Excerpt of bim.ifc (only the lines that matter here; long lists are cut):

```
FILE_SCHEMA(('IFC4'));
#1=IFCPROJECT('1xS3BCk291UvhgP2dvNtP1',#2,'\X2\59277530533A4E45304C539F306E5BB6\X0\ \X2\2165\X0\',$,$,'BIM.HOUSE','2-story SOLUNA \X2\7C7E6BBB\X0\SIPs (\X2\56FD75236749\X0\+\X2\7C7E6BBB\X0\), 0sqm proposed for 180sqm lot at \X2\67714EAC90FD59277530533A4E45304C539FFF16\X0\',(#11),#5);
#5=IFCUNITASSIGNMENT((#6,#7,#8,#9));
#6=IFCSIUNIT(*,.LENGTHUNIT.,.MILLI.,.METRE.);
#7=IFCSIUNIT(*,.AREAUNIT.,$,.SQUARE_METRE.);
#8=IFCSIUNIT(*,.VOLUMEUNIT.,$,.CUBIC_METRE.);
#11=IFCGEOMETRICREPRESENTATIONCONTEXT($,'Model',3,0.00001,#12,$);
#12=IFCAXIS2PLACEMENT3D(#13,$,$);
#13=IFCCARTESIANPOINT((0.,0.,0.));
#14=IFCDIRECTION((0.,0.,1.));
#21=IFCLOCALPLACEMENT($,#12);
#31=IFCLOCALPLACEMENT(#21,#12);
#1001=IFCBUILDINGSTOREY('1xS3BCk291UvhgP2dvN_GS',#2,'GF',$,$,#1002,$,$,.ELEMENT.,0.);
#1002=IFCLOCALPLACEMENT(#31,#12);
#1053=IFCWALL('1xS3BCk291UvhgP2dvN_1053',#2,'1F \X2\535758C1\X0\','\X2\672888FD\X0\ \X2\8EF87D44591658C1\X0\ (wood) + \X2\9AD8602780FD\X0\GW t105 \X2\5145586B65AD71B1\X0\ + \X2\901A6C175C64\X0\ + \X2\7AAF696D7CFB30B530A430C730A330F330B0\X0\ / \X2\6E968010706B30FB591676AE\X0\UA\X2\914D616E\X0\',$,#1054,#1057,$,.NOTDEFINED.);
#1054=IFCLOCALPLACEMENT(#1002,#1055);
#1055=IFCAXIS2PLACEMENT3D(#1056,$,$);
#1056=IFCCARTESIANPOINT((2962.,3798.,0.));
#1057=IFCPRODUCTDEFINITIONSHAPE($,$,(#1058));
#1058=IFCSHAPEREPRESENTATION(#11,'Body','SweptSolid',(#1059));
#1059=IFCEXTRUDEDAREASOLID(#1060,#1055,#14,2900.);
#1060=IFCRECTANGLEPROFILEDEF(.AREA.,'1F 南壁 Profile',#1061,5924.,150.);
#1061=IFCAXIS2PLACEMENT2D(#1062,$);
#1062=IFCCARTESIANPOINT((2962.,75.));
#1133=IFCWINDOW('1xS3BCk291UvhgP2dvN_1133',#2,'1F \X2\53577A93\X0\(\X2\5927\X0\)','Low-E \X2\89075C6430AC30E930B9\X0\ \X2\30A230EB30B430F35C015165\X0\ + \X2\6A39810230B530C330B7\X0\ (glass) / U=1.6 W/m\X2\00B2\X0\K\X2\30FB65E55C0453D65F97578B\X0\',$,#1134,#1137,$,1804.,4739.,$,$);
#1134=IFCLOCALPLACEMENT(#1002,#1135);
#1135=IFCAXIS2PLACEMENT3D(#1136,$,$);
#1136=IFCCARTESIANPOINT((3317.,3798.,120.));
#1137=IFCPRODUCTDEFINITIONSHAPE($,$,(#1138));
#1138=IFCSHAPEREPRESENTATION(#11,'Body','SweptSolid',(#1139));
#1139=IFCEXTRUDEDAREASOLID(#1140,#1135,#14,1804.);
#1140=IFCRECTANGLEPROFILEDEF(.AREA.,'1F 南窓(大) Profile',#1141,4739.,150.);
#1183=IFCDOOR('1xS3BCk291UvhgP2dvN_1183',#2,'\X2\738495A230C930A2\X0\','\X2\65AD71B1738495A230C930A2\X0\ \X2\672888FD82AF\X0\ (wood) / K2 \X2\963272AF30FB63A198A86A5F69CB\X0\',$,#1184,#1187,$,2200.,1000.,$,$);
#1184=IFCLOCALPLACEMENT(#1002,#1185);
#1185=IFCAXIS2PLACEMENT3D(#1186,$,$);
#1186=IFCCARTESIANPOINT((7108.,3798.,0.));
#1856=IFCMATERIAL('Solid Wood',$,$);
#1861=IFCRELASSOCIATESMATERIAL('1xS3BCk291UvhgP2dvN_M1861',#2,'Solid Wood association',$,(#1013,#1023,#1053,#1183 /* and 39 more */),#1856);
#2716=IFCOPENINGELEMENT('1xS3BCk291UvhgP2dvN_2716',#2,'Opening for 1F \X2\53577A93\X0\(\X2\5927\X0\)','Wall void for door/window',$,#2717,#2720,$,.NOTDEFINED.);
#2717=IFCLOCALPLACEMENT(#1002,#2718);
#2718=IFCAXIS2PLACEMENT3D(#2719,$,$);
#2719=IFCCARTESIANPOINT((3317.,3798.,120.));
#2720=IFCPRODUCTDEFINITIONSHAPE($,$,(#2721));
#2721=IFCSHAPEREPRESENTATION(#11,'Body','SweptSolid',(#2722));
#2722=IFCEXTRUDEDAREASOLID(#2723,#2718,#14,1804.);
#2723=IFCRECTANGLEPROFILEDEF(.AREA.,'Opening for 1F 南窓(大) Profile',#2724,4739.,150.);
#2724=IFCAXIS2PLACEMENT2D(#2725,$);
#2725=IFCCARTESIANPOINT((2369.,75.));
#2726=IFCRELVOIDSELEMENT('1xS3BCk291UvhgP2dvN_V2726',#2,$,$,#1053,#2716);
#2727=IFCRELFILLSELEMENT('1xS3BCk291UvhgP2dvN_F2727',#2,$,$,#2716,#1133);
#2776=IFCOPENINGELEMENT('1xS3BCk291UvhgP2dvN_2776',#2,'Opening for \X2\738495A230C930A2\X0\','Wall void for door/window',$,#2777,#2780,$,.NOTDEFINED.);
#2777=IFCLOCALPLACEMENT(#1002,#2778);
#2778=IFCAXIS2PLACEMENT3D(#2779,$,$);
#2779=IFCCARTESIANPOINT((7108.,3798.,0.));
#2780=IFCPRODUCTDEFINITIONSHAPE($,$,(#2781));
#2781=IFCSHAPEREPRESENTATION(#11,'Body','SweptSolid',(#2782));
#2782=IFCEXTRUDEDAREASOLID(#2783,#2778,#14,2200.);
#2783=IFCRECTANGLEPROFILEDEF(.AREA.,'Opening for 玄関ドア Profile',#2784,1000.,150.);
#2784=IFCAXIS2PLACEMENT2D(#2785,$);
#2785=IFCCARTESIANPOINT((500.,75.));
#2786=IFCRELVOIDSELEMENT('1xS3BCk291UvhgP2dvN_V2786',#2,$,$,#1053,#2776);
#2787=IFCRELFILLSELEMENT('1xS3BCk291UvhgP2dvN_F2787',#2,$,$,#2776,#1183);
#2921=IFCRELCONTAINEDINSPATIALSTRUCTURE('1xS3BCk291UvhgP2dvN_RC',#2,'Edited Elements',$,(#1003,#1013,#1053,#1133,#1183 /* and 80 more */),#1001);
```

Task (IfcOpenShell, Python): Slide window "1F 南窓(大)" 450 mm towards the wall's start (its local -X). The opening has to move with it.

```python
import ifcopenshell
import ifcopenshell.api.geometry
import ifcopenshell.util.placement
import ifcopenshell.util.unit

model = ifcopenshell.open("bim.ifc")
unit_scale = ifcopenshell.util.unit.calculate_unit_scale(model)

window = model.by_guid("1xS3BCk291UvhgP2dvN_1133")
opening = window.FillsVoids[0].RelatingOpeningElement
wall = opening.VoidsElements[0].RelatingBuildingElement

wall_matrix = ifcopenshell.util.placement.get_local_placement(wall.ObjectPlacement)
shift = wall_matrix[:3, 0] * -0.45 / unit_scale
before = ifcopenshell.util.placement.get_local_placement(window.ObjectPlacement)[:3, 3].copy()

# The window is not placed relative to its opening, so move both.
for product in (opening, window):
    matrix = ifcopenshell.util.placement.get_local_placement(product.ObjectPlacement)
    matrix[:3, 3] += shift
    ifcopenshell.api.geometry.edit_object_placement(model, product=product, matrix=matrix, is_si=False)

after = ifcopenshell.util.placement.get_local_placement(window.ObjectPlacement)[:3, 3]
print("window moved by", (after - before).round(3) + 0.0)

model.write("bim-out.ifc")
```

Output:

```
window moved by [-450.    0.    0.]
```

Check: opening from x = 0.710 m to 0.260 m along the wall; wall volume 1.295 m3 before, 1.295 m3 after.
